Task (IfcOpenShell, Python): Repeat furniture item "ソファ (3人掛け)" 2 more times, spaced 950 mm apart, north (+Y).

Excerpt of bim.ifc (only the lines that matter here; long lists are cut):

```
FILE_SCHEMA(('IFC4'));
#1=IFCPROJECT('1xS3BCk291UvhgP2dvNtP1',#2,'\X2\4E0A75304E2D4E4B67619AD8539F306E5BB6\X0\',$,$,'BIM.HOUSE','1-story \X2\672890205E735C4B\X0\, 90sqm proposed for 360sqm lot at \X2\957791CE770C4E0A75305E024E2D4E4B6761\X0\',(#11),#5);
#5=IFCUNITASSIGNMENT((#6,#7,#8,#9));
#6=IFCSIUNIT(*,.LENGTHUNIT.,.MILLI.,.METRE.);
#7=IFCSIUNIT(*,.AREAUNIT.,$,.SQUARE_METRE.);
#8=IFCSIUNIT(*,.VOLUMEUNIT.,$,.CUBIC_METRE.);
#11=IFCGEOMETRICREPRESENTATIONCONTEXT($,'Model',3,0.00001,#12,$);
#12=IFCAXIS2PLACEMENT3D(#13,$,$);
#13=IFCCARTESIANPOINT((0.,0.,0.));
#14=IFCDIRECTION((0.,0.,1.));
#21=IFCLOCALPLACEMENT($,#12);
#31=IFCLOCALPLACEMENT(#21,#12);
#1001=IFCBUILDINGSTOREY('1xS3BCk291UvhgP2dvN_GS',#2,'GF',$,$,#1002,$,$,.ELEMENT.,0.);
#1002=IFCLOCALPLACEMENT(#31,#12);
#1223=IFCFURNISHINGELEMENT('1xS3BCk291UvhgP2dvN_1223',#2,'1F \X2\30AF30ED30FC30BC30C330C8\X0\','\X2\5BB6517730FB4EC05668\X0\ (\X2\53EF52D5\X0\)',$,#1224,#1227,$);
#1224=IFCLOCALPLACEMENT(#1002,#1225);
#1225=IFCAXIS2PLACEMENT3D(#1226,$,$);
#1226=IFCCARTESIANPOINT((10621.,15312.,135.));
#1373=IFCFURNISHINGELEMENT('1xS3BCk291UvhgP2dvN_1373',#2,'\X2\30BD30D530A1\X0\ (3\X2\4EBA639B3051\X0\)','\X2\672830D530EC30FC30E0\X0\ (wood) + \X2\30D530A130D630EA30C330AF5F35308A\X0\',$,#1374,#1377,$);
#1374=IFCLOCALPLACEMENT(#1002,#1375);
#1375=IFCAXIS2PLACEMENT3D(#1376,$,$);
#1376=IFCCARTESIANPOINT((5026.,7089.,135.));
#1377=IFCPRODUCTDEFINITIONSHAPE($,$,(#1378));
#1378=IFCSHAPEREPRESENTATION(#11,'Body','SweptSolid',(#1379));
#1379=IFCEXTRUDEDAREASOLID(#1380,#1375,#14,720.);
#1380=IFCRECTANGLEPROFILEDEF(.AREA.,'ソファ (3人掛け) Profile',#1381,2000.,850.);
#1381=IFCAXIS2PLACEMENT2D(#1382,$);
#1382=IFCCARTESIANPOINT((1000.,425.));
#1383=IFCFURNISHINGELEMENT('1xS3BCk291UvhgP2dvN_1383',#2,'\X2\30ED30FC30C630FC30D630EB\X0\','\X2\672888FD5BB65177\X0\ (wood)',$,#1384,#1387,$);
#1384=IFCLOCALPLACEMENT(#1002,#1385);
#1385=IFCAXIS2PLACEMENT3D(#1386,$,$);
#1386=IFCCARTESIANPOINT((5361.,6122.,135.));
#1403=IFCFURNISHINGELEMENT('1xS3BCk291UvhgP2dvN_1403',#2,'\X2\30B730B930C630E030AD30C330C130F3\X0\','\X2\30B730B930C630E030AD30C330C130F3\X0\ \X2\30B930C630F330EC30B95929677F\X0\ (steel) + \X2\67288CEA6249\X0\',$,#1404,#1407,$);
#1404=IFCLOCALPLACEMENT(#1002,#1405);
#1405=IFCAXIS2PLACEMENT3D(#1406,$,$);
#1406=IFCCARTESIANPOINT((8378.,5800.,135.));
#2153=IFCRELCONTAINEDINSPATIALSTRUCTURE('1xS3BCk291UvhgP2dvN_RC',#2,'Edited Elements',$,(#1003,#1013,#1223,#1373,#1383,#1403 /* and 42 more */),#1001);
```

```python
import numpy as np
import ifcopenshell
import ifcopenshell.api.geometry
import ifcopenshell.api.root
import ifcopenshell.util.element
import ifcopenshell.util.placement
import ifcopenshell.util.unit

model = ifcopenshell.open("bim.ifc")
unit_scale = ifcopenshell.util.unit.calculate_unit_scale(model)


def reuse_history(source, copy):
    """copy_class also copies each property set's owner history, people and application; keep the originals."""
    for rel in copy.IsDefinedBy:
        if rel.is_a("IfcRelDefinesByProperties") and (history := rel.RelatingPropertyDefinition.OwnerHistory):
            rel.RelatingPropertyDefinition.OwnerHistory = source.OwnerHistory
            ifcopenshell.util.element.remove_deep2(model, history)


source = model.by_guid("1xS3BCk291UvhgP2dvN_1373")
base = ifcopenshell.util.placement.get_local_placement(source.ObjectPlacement)
step = np.array([0.0, 1.0, 0.0]) * 0.95 / unit_scale

for i in range(1, 3):
    copy = ifcopenshell.api.root.copy_class(model, product=source)
    copy.Representation = ifcopenshell.util.element.copy_deep(
        model, source.Representation, exclude=["IfcGeometricRepresentationContext", "IfcRepresentationMap"]
    )
    reuse_history(source, copy)
    matrix = base.copy()
    matrix[:3, 3] += i * step
    print("added at", matrix[:3, 3].round(3) + 0.0)
    ifcopenshell.api.geometry.edit_object_placement(model, product=copy, matrix=matrix, is_si=False)

model.write("bim_edited.ifc")
```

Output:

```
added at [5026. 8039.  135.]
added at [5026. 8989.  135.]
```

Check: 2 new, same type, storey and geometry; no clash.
